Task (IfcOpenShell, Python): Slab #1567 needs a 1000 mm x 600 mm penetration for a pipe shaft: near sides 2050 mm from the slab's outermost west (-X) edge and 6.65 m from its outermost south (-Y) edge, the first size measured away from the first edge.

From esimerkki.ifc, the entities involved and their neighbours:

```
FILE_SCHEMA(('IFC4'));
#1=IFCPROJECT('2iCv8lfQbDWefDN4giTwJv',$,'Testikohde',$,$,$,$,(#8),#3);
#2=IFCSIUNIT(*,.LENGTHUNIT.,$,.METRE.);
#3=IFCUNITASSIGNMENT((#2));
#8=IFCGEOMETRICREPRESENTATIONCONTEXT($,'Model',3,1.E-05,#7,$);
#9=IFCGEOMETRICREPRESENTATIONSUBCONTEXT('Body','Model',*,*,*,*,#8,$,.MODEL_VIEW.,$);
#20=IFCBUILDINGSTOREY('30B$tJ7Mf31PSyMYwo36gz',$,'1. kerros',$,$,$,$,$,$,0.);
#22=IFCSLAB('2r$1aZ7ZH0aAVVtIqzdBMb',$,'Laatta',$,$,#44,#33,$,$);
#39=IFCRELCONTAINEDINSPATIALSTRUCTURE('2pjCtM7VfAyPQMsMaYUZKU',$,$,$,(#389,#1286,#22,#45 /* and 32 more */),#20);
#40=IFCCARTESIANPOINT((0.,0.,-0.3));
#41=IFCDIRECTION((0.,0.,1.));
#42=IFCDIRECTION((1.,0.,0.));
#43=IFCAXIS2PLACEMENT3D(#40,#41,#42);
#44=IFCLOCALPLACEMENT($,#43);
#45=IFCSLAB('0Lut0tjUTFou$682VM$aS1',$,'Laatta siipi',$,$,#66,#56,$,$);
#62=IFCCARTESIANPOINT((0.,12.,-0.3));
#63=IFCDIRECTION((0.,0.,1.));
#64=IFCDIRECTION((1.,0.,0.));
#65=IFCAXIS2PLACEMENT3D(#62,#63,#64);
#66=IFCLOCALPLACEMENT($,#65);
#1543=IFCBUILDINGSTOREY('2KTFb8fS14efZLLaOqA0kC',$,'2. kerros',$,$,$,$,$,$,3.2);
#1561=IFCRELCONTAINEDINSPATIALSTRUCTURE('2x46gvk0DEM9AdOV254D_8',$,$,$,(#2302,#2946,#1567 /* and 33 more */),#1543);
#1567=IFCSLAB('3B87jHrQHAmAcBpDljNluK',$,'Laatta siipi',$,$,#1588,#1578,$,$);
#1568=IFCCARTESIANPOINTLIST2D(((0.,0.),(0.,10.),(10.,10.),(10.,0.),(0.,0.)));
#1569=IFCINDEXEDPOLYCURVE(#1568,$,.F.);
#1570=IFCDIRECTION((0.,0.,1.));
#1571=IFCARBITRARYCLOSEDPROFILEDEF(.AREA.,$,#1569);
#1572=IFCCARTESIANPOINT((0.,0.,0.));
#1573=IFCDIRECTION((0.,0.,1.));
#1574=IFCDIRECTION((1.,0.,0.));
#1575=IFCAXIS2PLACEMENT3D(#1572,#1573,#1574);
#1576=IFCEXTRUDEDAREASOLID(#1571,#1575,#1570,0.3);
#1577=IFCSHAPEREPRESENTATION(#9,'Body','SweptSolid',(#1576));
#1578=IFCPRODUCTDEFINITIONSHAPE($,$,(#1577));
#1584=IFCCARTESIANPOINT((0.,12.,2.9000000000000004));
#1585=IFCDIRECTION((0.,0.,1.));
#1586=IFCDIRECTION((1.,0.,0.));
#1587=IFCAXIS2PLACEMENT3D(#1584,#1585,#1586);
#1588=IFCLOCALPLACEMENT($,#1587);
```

```python
import numpy as np
import ifcopenshell
import ifcopenshell.api.feature
import ifcopenshell.api.geometry
import ifcopenshell.api.root
import ifcopenshell.geom
import ifcopenshell.util.placement
import ifcopenshell.util.representation
import ifcopenshell.util.shape
import ifcopenshell.util.unit

model = ifcopenshell.open("esimerkki.ifc")
unit_scale = ifcopenshell.util.unit.calculate_unit_scale(model)
settings = ifcopenshell.geom.settings()


def volume(element):
    """Net volume in cubic metres, openings subtracted."""
    shape = ifcopenshell.geom.create_shape(settings, element)
    return ifcopenshell.util.shape.get_volume(shape.geometry)


slab = model.by_id(1567)
before = volume(slab)

# Extent in the slab's own axes, in metres. The edges named are its -X and -Y sides.
slab_shape = ifcopenshell.geom.create_shape(settings, slab)
vertices = ifcopenshell.util.shape.get_vertices(slab_shape.geometry)
x_min, y_min, bottom = vertices.min(axis=0)
top = vertices[:, 2].max()

opening = ifcopenshell.api.root.create_entity(model, ifc_class="IfcOpeningElement", name="Pipe shaft opening", predefined_type="OPENING")
context = ifcopenshell.util.representation.get_context(model, "Model", "Body", "MODEL_VIEW")
width, depth = 1, 0.6
outline = [(0.0, 0.0), (width, 0.0), (width, depth), (0.0, depth), (0.0, 0.0)]
# Overshoot both faces by 50 mm so the cut is clean.
shape = ifcopenshell.api.geometry.add_slab_representation(
    model, context=context, depth=top - bottom + 0.1, polyline=outline
)
ifcopenshell.api.geometry.assign_representation(model, product=opening, representation=shape)

matrix = ifcopenshell.util.placement.get_local_placement(slab.ObjectPlacement)
matrix[:, 3] = matrix @ np.append(np.array([x_min + 2.05, y_min + 6.65, bottom - 0.05]) / unit_scale, 1.0)
ifcopenshell.api.geometry.edit_object_placement(model, product=opening, matrix=matrix, is_si=False)
ifcopenshell.api.feature.add_feature(model, feature=opening, element=slab)

after = volume(slab)

print(f"slab volume {before:.3f} -> {after:.3f} m3")

model.write("esimerkki_edited.ifc")
```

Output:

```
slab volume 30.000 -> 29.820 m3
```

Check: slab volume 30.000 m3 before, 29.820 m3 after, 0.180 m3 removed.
